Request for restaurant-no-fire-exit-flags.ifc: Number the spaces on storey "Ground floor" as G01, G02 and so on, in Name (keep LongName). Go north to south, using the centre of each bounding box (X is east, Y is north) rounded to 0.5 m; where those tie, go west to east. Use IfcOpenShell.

First a look at what the model holds.

```python
import ifcopenshell
import ifcopenshell.util.element
import ifcopenshell.util.placement

model = ifcopenshell.open("restaurant-no-fire-exit-flags.ifc")
print(model.schema)
storey = next(s for s in model.by_type("IfcBuildingStorey") if s.Name == "Ground floor")
spaces = [e for e in ifcopenshell.util.element.get_decomposition(storey) if e.is_a("IfcSpace")]
for e in sorted(spaces, key=lambda e: e.id()):
    origin = ifcopenshell.util.placement.get_local_placement(e.ObjectPlacement)[:3, 3]
    print(e.id(), e.Name, e.LongName, origin.round(2) + 0.0, sep=" | ")
```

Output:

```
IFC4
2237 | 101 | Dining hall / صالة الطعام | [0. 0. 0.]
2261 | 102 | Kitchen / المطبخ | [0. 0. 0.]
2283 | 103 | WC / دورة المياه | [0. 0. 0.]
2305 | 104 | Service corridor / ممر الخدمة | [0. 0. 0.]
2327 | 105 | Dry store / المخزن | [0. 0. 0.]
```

```python
import ifcopenshell
import ifcopenshell.geom
import ifcopenshell.util.element
import ifcopenshell.util.shape

model = ifcopenshell.open("restaurant-no-fire-exit-flags.ifc")
settings = ifcopenshell.geom.settings()
settings.set("use-world-coords", True)


def centre(element):
    shape = ifcopenshell.geom.create_shape(settings, element)
    return ifcopenshell.util.shape.get_bbox_centroid(shape.geometry)


storey = next(s for s in model.by_type("IfcBuildingStorey") if s.Name == "Ground floor")
spaces = [e for e in ifcopenshell.util.element.get_decomposition(storey) if e.is_a("IfcSpace")]

# Insertion points can sit at a corner or the storey origin, so sort by the geometry (in metres).
centres = {e: centre(e) for e in spaces}
spaces.sort(key=lambda e: (-round(centres[e][1] / 0.5), centres[e][0]))

for i, e in enumerate(spaces, start=1):
    number = f"G{i:02d}"
    e.Name = number
    print(e.id(), number)

model.write("restaurant-no-fire-exit-flags-out.ifc")
```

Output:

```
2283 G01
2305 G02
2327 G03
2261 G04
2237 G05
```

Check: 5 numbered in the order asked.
